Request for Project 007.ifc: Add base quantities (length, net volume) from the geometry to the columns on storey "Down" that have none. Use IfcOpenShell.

First a look at what the model holds.

```python
import ifcopenshell
import ifcopenshell.util.element
import ifcopenshell.util.unit

model = ifcopenshell.open("Project 007.ifc")
print(model.schema)
for unit_type in ("LENGTHUNIT", "AREAUNIT", "VOLUMEUNIT"):
    print(unit_type, ifcopenshell.util.unit.calculate_unit_scale(model, unit_type))
storey = next(s for s in model.by_type("IfcBuildingStorey") if s.Name == "Down")
columns = [e for e in ifcopenshell.util.element.get_decomposition(storey) if e.is_a("IfcColumn")]
for e in sorted(columns, key=lambda e: e.id()):
    print(e.id(), e.is_a(), e.Name, list(ifcopenshell.util.element.get_psets(e, qtos_only=True)), sep=" | ")
```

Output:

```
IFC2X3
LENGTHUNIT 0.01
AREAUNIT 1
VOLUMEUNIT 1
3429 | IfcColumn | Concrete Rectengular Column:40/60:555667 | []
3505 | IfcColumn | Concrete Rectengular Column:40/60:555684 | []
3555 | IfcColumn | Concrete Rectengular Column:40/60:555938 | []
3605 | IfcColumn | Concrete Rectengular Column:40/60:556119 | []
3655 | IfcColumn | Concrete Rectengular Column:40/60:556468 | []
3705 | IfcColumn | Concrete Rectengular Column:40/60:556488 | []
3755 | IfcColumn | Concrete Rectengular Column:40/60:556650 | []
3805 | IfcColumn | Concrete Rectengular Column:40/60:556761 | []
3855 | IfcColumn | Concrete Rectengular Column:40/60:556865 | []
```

```python
import ifcopenshell
import ifcopenshell.api.pset
import ifcopenshell.geom
import ifcopenshell.util.element
import ifcopenshell.util.shape
import ifcopenshell.util.unit

model = ifcopenshell.open("Project 007.ifc")
unit_scale = ifcopenshell.util.unit.calculate_unit_scale(model)
volume_scale = ifcopenshell.util.unit.calculate_unit_scale(model, "VOLUMEUNIT")
settings = ifcopenshell.geom.settings()

storey = next(s for s in model.by_type("IfcBuildingStorey") if s.Name == "Down")
columns = [e for e in ifcopenshell.util.element.get_decomposition(storey) if e.is_a("IfcColumn")]

for e in sorted(columns, key=lambda e: e.id()):
    if ifcopenshell.util.element.get_psets(e, qtos_only=True, should_inherit=False):
        continue
    # Geometry comes back in metres, in the element's own axes.
    shape = ifcopenshell.geom.create_shape(settings, e)
    values = {
        "Length": ifcopenshell.util.shape.get_z(shape.geometry) / unit_scale,
        "NetVolume": ifcopenshell.util.shape.get_volume(shape.geometry) / volume_scale,
    }
    qto = ifcopenshell.api.pset.add_qto(model, product=e, name="BaseQuantities")
    ifcopenshell.api.pset.edit_qto(model, qto=qto, properties=values)
    print(e.id(), {k: round(v, 3) for k, v in values.items()})

model.write("Project 007_rev.ifc")
```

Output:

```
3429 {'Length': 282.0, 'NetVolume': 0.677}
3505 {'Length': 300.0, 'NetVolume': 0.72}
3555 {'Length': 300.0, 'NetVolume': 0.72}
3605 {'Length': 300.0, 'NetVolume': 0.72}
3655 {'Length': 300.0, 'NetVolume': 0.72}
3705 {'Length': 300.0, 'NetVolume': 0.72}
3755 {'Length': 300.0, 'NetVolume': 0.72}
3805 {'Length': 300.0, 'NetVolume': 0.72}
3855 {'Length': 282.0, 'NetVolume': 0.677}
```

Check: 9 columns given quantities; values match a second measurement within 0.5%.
